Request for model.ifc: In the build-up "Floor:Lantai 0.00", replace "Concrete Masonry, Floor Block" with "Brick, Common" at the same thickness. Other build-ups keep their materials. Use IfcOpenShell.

First a look at what the model holds.

```python
import ifcopenshell
import ifcopenshell.util.element

model = ifcopenshell.open("model.ifc")
print(model.schema)
for layer_set in model.by_type("IfcMaterialLayerSet"):
    if layer_set.LayerSetName == "Floor:Lantai 0.00":
        for layer in layer_set.MaterialLayers:
            print(layer.id(), layer.Material and layer.Material.Name, layer.LayerThickness, sep=" | ")
        print(len(ifcopenshell.util.element.get_elements_by_material(model, layer_set)), "elements and types use it")
print(sorted(m.Name for m in model.by_type("IfcMaterial") if m.Name)[:60])
```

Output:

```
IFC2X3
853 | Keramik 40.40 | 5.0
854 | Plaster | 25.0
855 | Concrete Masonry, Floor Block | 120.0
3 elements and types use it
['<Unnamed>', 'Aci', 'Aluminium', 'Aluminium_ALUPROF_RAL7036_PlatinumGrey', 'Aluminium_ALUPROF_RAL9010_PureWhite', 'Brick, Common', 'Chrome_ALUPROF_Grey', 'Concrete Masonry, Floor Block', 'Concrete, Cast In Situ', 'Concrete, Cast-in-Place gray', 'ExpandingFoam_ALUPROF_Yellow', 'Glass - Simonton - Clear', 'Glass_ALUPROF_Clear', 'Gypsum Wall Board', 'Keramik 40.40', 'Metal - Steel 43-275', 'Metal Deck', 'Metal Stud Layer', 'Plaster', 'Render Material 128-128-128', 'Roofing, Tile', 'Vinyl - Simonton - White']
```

```python
import ifcopenshell
import ifcopenshell.api.material

model = ifcopenshell.open("model.ifc")

layer_set = next(s for s in model.by_type("IfcMaterialLayerSet") if s.LayerSetName == "Floor:Lantai 0.00")
layer = next(l for l in layer_set.MaterialLayers if l.Material and l.Material.Name == "Concrete Masonry, Floor Block")
material = next(m for m in model.by_type("IfcMaterial") if m.Name == "Brick, Common")

# Point this one layer at the other material; renaming the old one would change it everywhere.
ifcopenshell.api.material.edit_layer(model, layer=layer, attributes={}, material=material)

print([l.Material.Name if l.Material else None for l in layer_set.MaterialLayers])

model.write("model_edited.ifc")
```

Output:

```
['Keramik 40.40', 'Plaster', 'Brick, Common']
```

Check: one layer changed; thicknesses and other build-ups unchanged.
